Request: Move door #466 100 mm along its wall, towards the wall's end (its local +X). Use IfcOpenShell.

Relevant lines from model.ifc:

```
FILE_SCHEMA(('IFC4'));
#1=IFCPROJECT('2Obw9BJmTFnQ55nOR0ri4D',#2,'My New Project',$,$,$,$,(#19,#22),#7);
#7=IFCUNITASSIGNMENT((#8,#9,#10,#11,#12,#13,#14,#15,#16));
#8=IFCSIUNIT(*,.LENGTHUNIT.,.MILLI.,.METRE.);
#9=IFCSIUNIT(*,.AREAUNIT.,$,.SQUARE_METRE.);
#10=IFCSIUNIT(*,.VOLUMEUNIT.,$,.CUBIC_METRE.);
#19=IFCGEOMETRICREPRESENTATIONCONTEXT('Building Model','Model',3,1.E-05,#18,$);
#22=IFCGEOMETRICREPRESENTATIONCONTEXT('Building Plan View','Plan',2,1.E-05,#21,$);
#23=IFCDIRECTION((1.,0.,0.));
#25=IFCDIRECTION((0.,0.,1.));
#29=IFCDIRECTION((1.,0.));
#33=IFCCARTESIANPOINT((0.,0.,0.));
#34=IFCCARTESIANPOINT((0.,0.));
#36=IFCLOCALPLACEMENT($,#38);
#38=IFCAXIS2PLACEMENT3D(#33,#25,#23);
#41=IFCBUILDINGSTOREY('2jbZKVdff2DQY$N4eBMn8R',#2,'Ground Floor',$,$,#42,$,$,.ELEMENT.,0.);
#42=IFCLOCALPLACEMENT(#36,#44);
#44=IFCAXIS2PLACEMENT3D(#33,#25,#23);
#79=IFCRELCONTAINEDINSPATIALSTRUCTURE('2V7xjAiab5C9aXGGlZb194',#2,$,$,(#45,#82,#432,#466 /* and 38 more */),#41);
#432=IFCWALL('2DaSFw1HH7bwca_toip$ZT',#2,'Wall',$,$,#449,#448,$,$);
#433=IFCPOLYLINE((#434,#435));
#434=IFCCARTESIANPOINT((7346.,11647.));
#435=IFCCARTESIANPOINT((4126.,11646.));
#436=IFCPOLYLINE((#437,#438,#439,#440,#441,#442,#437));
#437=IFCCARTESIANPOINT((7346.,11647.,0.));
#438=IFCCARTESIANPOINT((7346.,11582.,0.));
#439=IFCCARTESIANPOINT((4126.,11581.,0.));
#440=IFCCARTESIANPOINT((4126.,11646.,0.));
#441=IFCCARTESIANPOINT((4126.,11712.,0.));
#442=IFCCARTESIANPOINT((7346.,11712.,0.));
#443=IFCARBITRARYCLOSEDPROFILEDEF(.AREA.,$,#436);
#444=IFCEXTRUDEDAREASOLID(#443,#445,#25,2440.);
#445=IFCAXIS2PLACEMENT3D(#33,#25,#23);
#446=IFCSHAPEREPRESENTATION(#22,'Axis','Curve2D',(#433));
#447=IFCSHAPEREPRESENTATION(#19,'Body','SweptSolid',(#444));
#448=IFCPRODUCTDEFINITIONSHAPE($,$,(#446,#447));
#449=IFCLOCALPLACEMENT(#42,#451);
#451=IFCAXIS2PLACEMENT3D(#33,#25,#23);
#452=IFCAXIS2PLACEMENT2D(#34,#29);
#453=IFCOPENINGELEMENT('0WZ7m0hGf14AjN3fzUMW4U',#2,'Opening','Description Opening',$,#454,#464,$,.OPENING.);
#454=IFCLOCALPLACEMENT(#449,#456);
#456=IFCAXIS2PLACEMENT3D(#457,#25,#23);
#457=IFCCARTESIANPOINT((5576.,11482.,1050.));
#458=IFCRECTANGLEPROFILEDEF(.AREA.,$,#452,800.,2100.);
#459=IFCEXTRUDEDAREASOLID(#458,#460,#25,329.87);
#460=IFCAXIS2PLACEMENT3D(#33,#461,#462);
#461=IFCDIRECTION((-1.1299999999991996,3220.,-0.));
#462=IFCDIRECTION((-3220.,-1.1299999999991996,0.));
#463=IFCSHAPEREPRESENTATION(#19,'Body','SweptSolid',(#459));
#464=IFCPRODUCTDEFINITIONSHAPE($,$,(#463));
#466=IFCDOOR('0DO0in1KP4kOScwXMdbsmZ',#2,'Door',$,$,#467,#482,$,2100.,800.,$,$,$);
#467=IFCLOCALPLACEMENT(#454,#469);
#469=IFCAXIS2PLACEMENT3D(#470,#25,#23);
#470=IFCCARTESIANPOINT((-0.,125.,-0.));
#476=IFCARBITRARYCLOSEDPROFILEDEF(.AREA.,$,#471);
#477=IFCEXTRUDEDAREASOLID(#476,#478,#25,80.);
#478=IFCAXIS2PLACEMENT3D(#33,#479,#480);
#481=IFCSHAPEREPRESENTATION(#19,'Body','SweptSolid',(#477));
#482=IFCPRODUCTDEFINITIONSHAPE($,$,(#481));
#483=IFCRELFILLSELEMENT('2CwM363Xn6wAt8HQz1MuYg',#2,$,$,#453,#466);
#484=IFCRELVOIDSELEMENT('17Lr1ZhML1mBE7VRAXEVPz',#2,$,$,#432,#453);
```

```python
import ifcopenshell
import ifcopenshell.api.geometry
import ifcopenshell.util.placement
import ifcopenshell.util.unit

model = ifcopenshell.open("model.ifc")
unit_scale = ifcopenshell.util.unit.calculate_unit_scale(model)

door = model.by_id(466)
opening = door.FillsVoids[0].RelatingOpeningElement
wall = opening.VoidsElements[0].RelatingBuildingElement

wall_matrix = ifcopenshell.util.placement.get_local_placement(wall.ObjectPlacement)
shift = wall_matrix[:3, 0] * 0.1 / unit_scale
before = ifcopenshell.util.placement.get_local_placement(door.ObjectPlacement)[:3, 3].copy()

# The door is placed relative to its opening, so it follows when the opening moves.
matrix = ifcopenshell.util.placement.get_local_placement(opening.ObjectPlacement)
matrix[:3, 3] += shift
ifcopenshell.api.geometry.edit_object_placement(
    model, product=opening, matrix=matrix, is_si=False, should_transform_children=True
)

after = ifcopenshell.util.placement.get_local_placement(door.ObjectPlacement)[:3, 3]
print("door moved by", (after - before).round(3) + 0.0)

model.write("model-out.ifc")
```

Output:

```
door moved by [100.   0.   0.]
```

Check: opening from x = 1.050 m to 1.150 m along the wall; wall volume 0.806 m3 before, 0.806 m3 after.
